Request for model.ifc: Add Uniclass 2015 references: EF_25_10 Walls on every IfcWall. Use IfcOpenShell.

First a look at what the model holds.

```python
import ifcopenshell

model = ifcopenshell.open("model.ifc")
print(model.schema)
print("classifications:", [c.Name for c in model.by_type("IfcClassification")])
for ifc_class in ("IfcDoor", "IfcRoof", "IfcStair", "IfcWall", "IfcWindow"):
    print(ifc_class, len(model.by_type(ifc_class)))
```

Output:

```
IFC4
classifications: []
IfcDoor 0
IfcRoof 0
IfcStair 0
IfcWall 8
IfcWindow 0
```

```python
import ifcopenshell
import ifcopenshell.api.classification

model = ifcopenshell.open("model.ifc")

system = ifcopenshell.api.classification.add_classification(model, classification="Uniclass 2015")

codes = {
    "IfcWall": ("EF_25_10", "Walls"),
}
for ifc_class, (code, name) in codes.items():
    products = model.by_type(ifc_class)
    ifcopenshell.api.classification.add_reference(
        model, products=products, classification=system, identification=code, name=name
    )
    print(code, len(products))

model.write("model-out.ifc")
```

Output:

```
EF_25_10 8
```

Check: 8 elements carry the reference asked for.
